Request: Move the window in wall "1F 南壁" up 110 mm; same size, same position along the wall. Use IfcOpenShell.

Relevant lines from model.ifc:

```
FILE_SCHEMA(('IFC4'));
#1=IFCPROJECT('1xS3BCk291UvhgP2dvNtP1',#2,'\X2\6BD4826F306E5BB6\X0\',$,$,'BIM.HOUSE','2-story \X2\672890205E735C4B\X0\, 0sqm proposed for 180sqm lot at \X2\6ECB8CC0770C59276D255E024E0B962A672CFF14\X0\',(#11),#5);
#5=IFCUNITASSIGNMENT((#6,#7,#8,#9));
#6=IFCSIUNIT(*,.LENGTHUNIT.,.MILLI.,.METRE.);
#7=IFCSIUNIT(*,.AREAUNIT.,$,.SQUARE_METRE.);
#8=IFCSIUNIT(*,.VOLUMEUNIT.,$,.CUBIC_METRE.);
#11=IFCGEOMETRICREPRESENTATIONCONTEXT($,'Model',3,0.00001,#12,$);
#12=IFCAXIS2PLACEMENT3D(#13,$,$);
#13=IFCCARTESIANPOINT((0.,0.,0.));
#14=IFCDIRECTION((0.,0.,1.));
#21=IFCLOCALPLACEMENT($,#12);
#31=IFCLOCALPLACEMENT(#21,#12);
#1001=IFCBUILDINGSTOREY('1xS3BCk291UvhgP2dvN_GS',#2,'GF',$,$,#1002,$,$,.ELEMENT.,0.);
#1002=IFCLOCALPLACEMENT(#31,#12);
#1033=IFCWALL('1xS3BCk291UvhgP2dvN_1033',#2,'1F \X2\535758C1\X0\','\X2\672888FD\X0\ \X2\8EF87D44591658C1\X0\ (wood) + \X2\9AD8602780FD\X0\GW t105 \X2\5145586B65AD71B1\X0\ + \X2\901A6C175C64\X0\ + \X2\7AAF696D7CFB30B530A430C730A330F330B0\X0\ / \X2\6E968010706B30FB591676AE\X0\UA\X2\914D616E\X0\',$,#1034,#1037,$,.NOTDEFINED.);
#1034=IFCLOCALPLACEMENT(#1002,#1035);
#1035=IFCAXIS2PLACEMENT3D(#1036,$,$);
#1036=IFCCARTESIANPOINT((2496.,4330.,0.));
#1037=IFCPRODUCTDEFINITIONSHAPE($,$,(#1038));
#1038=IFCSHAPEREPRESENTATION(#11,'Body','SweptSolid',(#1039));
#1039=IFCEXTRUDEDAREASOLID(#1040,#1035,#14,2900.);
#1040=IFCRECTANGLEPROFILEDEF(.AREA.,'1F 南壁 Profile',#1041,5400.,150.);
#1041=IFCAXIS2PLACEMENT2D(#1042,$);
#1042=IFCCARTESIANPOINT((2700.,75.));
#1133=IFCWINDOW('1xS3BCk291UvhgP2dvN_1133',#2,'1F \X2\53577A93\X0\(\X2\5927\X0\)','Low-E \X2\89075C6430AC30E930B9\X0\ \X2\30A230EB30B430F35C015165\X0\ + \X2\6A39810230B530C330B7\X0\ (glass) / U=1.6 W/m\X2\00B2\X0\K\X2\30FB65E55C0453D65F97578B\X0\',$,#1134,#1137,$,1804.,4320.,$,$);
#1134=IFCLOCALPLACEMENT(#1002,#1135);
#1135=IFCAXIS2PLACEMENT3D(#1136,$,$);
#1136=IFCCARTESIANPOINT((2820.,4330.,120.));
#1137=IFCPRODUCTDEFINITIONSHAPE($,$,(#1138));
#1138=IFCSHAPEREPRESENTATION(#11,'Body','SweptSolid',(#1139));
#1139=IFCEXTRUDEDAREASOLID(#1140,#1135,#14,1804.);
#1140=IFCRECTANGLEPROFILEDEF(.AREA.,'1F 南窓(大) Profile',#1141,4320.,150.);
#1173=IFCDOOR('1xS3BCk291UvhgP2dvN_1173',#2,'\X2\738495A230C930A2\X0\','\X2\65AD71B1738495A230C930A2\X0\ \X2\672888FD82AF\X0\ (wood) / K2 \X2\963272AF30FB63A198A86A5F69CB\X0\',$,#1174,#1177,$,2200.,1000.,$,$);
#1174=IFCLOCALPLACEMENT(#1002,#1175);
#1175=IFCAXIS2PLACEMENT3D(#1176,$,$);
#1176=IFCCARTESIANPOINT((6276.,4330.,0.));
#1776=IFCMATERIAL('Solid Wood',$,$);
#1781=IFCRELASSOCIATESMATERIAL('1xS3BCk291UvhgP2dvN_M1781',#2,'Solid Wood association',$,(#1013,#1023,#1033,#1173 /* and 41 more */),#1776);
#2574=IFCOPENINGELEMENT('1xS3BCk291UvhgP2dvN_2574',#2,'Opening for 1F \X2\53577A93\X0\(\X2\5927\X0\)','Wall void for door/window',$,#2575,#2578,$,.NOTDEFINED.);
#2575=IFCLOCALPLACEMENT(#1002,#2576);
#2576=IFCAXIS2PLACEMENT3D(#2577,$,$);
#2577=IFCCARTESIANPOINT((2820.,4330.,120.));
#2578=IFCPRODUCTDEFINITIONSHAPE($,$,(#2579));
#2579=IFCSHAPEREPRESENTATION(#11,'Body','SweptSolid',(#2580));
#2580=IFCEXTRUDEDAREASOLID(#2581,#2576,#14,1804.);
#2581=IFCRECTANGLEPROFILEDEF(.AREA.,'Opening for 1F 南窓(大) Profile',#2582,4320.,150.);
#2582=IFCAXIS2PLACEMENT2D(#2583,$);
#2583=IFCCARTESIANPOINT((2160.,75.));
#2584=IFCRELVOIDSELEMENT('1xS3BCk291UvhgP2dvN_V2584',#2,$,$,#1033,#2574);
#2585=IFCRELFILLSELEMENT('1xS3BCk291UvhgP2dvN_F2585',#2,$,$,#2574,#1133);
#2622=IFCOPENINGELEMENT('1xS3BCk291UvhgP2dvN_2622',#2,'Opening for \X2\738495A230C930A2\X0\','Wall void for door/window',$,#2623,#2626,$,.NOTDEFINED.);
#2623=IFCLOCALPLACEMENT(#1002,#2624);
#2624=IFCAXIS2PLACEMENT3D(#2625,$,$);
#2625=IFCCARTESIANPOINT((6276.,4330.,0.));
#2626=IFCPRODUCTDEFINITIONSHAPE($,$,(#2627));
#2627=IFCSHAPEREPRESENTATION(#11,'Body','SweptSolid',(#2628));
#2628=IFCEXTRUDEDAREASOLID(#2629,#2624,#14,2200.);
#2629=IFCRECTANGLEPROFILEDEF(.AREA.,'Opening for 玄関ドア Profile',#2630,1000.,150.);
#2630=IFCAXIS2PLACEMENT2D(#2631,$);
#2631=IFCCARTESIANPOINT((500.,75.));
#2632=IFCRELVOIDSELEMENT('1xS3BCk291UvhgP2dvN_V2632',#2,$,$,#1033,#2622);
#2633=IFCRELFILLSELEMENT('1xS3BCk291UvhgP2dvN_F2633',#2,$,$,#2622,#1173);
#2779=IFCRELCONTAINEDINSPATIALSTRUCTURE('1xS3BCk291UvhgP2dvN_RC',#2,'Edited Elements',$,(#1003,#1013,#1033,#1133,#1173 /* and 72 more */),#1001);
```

```python
import numpy as np
import ifcopenshell
import ifcopenshell.api.geometry
import ifcopenshell.util.placement
import ifcopenshell.util.unit

model = ifcopenshell.open("model.ifc")
unit_scale = ifcopenshell.util.unit.calculate_unit_scale(model)

window = model.by_guid("1xS3BCk291UvhgP2dvN_1133")
opening = window.FillsVoids[0].RelatingOpeningElement
dz = 0.11 / unit_scale

shift = np.array([0.0, 0.0, dz])
# The window is not placed relative to its opening, so move both.
for product in (opening, window):
    matrix = ifcopenshell.util.placement.get_local_placement(product.ObjectPlacement)
    matrix[:3, 3] += shift
    ifcopenshell.api.geometry.edit_object_placement(model, product=product, matrix=matrix, is_si=False)

print(f"moved by {dz * unit_scale:+.3f} m")

model.write("model_edited.ifc")
```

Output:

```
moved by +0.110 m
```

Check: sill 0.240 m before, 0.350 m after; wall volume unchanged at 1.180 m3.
